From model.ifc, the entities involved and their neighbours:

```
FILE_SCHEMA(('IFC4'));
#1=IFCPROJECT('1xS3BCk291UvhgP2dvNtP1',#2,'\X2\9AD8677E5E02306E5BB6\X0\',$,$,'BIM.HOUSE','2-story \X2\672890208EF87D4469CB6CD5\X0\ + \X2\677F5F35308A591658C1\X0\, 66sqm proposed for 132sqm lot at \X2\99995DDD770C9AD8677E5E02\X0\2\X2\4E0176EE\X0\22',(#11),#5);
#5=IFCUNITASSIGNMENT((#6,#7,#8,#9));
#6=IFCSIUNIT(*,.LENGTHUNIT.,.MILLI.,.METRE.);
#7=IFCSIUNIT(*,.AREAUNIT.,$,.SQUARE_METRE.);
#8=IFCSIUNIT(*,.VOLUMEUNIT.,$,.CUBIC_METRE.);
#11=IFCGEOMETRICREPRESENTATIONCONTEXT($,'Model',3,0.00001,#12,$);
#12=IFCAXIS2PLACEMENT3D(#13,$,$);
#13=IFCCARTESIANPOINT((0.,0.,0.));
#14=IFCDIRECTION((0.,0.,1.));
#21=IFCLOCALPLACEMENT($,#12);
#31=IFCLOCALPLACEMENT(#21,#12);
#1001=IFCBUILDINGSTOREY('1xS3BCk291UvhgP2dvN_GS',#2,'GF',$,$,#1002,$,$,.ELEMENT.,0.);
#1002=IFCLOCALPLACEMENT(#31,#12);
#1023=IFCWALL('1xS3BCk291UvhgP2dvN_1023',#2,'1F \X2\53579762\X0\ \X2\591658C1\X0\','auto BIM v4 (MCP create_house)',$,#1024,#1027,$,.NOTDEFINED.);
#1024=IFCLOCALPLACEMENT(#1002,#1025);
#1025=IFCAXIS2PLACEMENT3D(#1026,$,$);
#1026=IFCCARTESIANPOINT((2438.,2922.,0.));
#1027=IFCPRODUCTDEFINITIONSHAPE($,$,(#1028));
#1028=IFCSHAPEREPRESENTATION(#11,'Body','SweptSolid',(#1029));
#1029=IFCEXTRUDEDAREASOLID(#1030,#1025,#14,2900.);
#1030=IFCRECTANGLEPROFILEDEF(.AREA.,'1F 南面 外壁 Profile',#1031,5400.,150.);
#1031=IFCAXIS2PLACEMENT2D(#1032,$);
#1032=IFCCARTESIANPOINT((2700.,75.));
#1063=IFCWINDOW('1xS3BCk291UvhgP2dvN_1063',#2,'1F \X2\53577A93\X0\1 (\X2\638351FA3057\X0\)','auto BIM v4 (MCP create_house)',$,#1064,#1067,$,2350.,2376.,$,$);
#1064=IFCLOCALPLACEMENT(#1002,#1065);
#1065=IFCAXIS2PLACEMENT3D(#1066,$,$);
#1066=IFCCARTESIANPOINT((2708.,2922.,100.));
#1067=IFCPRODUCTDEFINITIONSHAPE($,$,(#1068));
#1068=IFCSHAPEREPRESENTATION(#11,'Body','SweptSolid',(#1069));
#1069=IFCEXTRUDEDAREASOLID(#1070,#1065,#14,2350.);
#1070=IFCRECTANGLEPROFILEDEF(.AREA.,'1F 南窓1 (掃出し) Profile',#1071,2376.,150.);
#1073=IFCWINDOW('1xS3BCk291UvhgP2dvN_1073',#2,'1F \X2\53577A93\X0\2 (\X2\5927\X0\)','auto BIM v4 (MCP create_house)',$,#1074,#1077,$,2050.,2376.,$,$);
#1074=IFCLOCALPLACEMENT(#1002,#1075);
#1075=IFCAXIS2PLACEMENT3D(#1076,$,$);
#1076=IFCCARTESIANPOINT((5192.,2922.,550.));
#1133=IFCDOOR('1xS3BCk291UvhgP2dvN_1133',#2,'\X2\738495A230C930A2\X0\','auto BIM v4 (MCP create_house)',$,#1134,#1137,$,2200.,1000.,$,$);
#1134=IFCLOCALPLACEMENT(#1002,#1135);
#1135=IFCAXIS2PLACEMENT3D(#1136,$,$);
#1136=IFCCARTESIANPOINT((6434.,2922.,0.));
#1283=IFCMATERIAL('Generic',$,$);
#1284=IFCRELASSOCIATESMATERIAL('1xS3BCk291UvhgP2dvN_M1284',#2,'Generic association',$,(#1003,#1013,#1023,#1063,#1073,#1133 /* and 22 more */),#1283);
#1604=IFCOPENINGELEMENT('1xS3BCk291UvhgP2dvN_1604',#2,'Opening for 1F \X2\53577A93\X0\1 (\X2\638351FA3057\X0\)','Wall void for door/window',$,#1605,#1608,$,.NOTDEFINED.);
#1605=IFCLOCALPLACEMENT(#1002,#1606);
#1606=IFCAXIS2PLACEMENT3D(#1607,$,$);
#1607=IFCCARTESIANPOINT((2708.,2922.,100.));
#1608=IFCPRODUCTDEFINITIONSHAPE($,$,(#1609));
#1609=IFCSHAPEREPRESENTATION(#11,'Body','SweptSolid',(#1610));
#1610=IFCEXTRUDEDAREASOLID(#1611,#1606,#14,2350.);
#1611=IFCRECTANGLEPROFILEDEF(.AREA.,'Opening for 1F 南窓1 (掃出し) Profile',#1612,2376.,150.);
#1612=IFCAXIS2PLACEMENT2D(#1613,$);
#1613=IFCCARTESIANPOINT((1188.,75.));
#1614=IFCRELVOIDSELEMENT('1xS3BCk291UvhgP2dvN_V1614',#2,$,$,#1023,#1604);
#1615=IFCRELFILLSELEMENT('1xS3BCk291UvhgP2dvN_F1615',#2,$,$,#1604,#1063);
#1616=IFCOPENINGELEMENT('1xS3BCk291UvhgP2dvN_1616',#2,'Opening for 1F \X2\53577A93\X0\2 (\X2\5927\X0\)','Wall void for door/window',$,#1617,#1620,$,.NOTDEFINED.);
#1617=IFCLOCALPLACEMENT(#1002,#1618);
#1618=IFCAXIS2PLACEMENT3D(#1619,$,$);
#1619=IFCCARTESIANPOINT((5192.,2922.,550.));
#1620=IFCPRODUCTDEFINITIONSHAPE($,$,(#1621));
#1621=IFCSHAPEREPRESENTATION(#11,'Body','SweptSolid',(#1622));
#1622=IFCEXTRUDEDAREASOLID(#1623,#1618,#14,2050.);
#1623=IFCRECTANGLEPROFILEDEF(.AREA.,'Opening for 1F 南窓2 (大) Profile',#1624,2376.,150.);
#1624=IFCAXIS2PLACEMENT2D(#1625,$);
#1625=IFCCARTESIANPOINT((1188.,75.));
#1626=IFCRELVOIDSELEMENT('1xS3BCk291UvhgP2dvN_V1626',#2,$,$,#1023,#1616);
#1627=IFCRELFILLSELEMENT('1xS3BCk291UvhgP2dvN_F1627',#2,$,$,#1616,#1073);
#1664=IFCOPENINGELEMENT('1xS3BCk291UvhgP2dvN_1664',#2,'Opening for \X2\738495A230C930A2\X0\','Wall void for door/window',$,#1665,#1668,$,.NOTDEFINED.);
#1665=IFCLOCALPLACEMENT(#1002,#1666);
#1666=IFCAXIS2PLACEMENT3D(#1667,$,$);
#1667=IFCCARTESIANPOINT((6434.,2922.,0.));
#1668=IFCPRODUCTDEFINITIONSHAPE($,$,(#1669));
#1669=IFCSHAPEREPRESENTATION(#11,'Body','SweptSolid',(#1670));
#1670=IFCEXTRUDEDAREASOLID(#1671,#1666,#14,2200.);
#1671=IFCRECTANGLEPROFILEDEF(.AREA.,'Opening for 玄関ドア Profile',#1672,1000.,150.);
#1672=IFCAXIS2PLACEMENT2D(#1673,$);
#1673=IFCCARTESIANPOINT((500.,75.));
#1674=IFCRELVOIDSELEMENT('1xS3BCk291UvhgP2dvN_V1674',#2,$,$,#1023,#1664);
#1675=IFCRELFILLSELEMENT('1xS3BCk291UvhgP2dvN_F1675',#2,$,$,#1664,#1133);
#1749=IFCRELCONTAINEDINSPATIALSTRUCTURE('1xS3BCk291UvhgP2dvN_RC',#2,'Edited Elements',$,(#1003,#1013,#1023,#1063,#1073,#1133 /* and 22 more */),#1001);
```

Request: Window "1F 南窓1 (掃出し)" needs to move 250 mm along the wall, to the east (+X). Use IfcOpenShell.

```python
import ifcopenshell
import ifcopenshell.api.geometry
import ifcopenshell.util.placement
import ifcopenshell.util.unit

model = ifcopenshell.open("model.ifc")
unit_scale = ifcopenshell.util.unit.calculate_unit_scale(model)

window = model.by_guid("1xS3BCk291UvhgP2dvN_1063")
opening = window.FillsVoids[0].RelatingOpeningElement
wall = opening.VoidsElements[0].RelatingBuildingElement

wall_matrix = ifcopenshell.util.placement.get_local_placement(wall.ObjectPlacement)
shift = wall_matrix[:3, 0] * 0.25 / unit_scale
before = ifcopenshell.util.placement.get_local_placement(window.ObjectPlacement)[:3, 3].copy()

# The window is not placed relative to its opening, so move both.
for product in (opening, window):
    matrix = ifcopenshell.util.placement.get_local_placement(product.ObjectPlacement)
    matrix[:3, 3] += shift
    ifcopenshell.api.geometry.edit_object_placement(model, product=product, matrix=matrix, is_si=False)

after = ifcopenshell.util.placement.get_local_placement(window.ObjectPlacement)[:3, 3]
print("window moved by", (after - before).round(3) + 0.0)

model.write("model_rev.ifc")
```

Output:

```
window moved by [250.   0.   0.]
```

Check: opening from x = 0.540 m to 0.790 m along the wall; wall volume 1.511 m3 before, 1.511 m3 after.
